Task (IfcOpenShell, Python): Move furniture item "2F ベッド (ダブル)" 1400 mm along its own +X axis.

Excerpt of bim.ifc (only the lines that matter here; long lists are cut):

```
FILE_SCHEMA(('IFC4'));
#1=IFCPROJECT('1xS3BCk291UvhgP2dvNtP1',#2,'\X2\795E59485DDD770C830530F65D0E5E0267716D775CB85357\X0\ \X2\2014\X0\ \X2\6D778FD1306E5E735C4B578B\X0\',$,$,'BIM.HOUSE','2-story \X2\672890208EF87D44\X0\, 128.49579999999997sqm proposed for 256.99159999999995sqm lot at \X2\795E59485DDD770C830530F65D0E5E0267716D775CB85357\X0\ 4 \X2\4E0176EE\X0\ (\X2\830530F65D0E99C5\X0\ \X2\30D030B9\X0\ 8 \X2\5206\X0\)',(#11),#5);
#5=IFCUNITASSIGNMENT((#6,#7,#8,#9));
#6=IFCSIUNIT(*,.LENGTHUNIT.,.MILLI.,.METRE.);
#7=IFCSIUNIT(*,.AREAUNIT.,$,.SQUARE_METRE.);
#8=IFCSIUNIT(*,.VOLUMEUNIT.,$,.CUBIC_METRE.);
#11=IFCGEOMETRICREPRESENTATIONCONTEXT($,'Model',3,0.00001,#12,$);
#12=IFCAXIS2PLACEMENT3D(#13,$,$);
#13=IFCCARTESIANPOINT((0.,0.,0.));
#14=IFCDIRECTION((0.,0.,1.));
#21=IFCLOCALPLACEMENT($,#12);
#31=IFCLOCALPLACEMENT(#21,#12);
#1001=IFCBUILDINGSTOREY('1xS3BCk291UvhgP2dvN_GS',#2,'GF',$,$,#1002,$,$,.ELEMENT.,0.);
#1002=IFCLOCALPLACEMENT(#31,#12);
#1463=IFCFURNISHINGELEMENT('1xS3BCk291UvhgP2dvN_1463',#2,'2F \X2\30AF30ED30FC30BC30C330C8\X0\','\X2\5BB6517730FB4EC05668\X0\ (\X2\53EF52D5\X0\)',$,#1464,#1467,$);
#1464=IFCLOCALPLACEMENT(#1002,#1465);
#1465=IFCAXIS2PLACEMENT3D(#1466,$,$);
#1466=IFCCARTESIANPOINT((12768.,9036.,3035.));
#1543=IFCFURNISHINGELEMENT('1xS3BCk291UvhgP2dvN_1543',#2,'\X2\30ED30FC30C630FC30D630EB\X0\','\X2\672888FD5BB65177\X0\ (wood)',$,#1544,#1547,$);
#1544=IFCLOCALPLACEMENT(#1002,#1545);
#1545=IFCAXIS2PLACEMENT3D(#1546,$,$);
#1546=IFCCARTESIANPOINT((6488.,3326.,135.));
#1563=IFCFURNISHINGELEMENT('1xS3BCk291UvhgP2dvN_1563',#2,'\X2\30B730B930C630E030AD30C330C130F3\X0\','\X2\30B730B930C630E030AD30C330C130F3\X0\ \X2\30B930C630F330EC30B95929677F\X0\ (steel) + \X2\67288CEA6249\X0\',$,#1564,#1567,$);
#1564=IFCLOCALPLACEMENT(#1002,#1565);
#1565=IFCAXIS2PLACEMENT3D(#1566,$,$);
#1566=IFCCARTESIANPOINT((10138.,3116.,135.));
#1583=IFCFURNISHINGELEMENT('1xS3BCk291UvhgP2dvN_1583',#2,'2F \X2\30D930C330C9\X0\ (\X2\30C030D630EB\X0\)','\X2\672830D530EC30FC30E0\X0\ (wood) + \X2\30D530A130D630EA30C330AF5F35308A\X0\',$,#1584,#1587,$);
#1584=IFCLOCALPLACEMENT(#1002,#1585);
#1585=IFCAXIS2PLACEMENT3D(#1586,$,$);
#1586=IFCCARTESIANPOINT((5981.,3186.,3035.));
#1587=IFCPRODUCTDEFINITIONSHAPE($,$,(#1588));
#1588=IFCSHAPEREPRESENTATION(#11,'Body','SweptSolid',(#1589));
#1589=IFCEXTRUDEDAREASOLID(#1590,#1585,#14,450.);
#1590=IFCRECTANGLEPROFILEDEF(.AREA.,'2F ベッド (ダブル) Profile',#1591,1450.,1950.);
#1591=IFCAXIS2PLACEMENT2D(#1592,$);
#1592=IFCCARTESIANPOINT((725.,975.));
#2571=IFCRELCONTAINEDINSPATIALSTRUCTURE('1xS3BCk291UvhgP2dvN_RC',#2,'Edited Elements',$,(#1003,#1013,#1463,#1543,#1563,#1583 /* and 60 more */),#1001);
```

```python
import ifcopenshell
import ifcopenshell.api.geometry
import ifcopenshell.util.placement
import ifcopenshell.util.unit

model = ifcopenshell.open("bim.ifc")
unit_scale = ifcopenshell.util.unit.calculate_unit_scale(model)

item = model.by_guid("1xS3BCk291UvhgP2dvN_1583")
matrix = ifcopenshell.util.placement.get_local_placement(item.ObjectPlacement)
matrix[:3, 3] += matrix[:3, 0] * 1.4 / unit_scale
ifcopenshell.api.geometry.edit_object_placement(model, product=item, matrix=matrix, is_si=False)

print(ifcopenshell.util.placement.get_local_placement(item.ObjectPlacement).round(3) + 0.0)

model.write("bim_v2.ifc")
```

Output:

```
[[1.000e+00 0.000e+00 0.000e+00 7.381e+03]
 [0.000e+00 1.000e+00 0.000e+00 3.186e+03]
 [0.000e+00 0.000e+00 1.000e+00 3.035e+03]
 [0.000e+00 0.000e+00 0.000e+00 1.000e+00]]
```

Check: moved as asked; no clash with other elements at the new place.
